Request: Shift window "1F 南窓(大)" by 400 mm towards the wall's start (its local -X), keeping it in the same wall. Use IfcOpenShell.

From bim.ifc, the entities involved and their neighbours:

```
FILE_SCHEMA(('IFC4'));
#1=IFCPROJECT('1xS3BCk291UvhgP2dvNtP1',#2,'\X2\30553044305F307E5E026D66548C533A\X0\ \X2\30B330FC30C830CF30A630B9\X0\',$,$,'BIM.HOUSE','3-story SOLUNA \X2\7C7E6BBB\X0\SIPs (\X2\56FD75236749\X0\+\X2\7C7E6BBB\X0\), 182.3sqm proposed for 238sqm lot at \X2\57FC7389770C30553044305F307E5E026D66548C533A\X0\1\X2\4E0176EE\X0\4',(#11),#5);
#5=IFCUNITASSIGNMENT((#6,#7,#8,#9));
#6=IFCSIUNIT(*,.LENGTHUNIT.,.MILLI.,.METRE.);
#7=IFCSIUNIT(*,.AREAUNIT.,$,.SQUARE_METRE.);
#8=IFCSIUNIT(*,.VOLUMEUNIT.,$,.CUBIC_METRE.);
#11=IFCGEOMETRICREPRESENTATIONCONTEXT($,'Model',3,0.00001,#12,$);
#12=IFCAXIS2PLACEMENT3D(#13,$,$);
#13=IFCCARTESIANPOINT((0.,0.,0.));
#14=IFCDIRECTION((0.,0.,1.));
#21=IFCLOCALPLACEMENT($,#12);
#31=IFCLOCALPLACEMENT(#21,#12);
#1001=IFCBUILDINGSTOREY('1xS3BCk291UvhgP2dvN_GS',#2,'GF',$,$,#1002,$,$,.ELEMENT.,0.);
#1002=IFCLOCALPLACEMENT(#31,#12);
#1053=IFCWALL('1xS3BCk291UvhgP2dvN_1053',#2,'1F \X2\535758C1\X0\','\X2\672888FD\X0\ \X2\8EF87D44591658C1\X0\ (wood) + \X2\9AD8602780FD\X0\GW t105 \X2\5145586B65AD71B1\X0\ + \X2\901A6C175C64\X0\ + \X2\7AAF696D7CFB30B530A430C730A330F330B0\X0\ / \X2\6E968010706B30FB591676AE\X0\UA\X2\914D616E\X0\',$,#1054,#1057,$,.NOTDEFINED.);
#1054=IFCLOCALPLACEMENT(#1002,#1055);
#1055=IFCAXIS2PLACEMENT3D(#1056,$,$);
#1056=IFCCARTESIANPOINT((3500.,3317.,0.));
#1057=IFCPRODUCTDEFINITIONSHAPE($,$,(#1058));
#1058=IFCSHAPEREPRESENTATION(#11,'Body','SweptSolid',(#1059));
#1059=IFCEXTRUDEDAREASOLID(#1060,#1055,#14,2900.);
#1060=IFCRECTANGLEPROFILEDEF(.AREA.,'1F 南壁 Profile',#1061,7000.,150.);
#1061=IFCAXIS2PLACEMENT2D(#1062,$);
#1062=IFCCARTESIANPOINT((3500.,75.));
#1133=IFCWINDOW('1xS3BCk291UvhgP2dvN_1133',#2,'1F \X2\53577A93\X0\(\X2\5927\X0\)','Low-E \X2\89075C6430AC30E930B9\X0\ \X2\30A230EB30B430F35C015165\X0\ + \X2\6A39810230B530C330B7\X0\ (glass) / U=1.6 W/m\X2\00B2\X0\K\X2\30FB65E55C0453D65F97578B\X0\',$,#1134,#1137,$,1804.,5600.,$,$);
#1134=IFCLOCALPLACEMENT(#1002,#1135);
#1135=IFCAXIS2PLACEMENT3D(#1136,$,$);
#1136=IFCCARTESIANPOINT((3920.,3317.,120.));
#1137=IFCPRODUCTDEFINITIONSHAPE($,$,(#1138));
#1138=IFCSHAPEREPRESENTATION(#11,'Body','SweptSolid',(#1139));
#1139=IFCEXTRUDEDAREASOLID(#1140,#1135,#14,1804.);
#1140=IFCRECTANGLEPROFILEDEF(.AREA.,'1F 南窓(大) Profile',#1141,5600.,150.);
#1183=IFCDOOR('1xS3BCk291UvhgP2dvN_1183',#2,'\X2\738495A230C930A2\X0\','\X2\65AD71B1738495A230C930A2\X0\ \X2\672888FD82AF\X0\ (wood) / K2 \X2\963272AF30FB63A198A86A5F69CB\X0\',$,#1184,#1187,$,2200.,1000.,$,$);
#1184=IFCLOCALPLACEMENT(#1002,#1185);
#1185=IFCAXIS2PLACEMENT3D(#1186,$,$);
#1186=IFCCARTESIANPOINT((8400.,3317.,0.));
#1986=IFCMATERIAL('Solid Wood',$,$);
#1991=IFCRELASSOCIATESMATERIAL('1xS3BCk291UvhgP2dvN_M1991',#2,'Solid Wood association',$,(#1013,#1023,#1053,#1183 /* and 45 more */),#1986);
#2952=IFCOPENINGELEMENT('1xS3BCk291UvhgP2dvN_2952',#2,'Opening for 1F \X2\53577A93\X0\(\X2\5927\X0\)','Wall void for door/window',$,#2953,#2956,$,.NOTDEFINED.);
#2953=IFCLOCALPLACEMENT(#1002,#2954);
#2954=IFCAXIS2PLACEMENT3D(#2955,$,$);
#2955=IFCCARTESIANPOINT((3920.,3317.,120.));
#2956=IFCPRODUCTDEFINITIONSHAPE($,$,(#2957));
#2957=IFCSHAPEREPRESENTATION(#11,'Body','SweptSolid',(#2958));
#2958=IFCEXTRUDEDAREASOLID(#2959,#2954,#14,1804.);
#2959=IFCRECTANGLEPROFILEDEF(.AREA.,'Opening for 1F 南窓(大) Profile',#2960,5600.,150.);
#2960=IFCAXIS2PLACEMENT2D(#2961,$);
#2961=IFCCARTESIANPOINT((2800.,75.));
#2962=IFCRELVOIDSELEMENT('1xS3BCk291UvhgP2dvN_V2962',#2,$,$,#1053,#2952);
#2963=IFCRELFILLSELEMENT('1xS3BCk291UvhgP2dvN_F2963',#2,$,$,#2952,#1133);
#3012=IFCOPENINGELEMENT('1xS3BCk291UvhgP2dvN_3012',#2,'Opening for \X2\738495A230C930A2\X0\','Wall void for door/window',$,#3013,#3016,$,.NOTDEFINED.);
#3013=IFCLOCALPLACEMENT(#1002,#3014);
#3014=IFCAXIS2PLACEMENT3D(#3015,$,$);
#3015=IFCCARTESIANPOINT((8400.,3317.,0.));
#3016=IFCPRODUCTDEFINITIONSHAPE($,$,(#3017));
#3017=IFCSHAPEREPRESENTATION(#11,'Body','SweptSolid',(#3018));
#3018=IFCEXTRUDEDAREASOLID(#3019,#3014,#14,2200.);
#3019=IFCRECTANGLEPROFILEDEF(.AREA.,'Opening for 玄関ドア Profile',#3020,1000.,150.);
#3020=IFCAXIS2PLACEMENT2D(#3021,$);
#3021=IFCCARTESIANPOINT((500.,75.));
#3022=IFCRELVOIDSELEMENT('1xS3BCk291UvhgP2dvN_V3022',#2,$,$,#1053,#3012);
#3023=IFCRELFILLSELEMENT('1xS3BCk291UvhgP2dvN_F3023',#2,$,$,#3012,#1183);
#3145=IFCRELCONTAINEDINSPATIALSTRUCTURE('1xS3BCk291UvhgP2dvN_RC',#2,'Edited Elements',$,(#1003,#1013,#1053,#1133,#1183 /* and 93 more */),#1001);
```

```python
import ifcopenshell
import ifcopenshell.api.geometry
import ifcopenshell.util.placement
import ifcopenshell.util.unit

model = ifcopenshell.open("bim.ifc")
unit_scale = ifcopenshell.util.unit.calculate_unit_scale(model)

window = model.by_guid("1xS3BCk291UvhgP2dvN_1133")
opening = window.FillsVoids[0].RelatingOpeningElement
wall = opening.VoidsElements[0].RelatingBuildingElement

wall_matrix = ifcopenshell.util.placement.get_local_placement(wall.ObjectPlacement)
shift = wall_matrix[:3, 0] * -0.4 / unit_scale
before = ifcopenshell.util.placement.get_local_placement(window.ObjectPlacement)[:3, 3].copy()

# The window is not placed relative to its opening, so move both.
for product in (opening, window):
    matrix = ifcopenshell.util.placement.get_local_placement(product.ObjectPlacement)
    matrix[:3, 3] += shift
    ifcopenshell.api.geometry.edit_object_placement(model, product=product, matrix=matrix, is_si=False)

after = ifcopenshell.util.placement.get_local_placement(window.ObjectPlacement)[:3, 3]
print("window moved by", (after - before).round(3) + 0.0)

model.write("bim_updated.ifc")
```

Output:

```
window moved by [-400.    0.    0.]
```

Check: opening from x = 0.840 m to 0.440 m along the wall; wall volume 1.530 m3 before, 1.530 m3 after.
